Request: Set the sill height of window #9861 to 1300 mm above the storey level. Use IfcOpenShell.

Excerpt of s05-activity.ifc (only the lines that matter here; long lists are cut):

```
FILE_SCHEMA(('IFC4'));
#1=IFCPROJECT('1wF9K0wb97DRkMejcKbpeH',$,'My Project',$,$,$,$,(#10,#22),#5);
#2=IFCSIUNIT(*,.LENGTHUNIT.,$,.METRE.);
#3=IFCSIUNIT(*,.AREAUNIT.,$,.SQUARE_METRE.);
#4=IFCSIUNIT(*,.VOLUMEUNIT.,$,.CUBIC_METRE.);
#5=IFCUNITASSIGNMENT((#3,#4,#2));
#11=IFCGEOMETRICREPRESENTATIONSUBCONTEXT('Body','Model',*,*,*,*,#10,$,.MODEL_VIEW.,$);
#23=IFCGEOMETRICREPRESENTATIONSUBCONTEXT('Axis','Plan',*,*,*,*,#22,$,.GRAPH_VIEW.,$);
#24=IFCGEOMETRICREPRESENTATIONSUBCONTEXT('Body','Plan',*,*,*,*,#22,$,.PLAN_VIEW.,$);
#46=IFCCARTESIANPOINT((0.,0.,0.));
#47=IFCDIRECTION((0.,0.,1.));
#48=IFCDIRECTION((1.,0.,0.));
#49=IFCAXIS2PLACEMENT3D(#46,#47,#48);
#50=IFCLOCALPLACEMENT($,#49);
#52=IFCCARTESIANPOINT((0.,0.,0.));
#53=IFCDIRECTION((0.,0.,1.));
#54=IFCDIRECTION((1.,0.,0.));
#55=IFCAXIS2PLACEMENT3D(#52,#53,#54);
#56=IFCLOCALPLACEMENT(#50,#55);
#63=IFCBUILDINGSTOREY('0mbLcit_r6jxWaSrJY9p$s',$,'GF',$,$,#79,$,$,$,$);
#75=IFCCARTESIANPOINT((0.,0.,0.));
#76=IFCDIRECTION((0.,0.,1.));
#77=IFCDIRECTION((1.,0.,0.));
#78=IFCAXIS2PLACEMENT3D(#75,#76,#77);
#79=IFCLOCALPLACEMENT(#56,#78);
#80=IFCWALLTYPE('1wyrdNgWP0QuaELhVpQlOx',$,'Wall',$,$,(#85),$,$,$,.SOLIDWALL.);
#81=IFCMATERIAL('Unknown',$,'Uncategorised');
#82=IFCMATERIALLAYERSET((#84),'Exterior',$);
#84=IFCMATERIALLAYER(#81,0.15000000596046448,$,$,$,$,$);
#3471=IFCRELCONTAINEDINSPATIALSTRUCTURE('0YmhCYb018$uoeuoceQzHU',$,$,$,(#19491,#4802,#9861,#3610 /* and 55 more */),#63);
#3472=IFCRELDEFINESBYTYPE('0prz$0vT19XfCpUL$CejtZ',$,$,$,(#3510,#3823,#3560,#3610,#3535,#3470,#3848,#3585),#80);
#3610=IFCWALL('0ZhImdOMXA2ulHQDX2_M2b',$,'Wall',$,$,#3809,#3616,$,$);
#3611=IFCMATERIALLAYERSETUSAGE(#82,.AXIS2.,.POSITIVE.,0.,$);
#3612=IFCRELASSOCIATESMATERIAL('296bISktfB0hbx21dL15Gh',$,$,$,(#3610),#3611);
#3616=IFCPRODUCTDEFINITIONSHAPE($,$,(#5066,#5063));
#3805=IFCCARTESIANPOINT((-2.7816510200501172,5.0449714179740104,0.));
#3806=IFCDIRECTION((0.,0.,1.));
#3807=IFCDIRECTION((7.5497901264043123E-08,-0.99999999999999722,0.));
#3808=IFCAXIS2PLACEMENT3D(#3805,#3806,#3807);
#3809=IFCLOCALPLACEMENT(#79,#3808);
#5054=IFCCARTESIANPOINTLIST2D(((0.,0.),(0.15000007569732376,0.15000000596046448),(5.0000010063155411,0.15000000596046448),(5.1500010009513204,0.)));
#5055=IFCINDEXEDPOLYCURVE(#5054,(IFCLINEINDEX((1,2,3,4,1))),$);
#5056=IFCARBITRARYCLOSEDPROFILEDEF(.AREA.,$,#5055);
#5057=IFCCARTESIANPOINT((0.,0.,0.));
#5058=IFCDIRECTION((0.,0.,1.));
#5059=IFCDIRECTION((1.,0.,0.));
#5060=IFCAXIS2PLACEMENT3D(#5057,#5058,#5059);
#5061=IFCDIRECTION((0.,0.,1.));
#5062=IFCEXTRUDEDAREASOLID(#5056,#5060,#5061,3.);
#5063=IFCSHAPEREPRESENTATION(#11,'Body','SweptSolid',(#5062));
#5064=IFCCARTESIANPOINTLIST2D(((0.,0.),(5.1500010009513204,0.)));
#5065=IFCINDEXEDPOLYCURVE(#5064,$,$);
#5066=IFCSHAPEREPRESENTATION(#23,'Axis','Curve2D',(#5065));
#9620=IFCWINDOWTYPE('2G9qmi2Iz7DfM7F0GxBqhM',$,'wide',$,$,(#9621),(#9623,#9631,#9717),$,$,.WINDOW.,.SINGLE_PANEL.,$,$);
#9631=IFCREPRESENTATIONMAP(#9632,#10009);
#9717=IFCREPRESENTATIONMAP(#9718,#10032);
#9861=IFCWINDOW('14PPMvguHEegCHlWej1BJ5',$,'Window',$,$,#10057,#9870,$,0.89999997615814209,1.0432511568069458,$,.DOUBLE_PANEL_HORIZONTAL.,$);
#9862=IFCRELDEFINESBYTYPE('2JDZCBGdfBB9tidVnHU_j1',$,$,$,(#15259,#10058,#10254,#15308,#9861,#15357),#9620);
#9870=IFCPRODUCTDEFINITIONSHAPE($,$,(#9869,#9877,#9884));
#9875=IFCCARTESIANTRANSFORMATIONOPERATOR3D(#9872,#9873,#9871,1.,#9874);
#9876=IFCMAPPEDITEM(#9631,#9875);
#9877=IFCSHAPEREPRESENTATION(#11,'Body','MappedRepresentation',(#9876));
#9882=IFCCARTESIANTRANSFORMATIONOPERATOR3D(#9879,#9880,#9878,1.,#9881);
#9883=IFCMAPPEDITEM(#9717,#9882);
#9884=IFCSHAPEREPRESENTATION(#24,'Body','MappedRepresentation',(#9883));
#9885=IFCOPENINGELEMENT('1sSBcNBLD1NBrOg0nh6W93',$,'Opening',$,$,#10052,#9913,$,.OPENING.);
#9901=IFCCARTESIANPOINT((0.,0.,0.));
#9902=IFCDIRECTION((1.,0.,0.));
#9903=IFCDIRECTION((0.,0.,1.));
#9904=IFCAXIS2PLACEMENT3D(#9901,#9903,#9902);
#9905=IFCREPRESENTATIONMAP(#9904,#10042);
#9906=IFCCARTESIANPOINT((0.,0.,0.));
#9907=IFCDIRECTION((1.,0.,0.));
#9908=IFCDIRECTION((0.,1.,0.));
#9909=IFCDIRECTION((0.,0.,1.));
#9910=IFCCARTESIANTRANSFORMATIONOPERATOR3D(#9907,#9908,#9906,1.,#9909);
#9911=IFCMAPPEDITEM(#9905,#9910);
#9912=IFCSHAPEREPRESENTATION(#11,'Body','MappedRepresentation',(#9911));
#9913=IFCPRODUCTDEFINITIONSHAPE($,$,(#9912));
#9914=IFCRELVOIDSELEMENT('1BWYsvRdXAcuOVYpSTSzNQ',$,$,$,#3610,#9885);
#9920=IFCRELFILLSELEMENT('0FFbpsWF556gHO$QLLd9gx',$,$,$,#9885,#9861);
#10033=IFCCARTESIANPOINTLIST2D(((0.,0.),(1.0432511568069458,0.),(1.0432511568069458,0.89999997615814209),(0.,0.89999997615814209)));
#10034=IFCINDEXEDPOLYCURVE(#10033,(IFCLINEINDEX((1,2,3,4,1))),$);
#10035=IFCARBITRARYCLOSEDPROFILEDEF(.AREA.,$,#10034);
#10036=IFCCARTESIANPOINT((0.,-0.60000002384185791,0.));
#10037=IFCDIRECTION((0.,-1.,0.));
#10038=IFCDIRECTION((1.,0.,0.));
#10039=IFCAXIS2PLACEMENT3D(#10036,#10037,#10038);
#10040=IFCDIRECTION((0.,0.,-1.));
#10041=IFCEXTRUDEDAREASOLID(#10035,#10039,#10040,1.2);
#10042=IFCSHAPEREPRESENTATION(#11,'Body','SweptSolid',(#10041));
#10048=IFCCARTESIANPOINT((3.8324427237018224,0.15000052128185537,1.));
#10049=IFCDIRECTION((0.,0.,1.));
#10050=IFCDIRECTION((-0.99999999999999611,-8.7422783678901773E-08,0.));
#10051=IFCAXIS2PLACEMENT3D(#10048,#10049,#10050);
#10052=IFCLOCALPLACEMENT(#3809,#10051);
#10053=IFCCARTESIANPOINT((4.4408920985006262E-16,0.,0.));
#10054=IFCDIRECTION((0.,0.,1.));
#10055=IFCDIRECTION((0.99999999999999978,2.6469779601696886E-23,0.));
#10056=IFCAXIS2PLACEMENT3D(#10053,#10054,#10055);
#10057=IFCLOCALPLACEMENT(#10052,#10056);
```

```python
import numpy as np
import ifcopenshell
import ifcopenshell.api.geometry
import ifcopenshell.geom
import ifcopenshell.util.element
import ifcopenshell.util.placement
import ifcopenshell.util.shape
import ifcopenshell.util.unit

model = ifcopenshell.open("s05-activity.ifc")
unit_scale = ifcopenshell.util.unit.calculate_unit_scale(model)

window = model.by_guid("14PPMvguHEegCHlWej1BJ5")
opening = window.FillsVoids[0].RelatingOpeningElement
storey = ifcopenshell.util.element.get_container(window, ifc_class="IfcBuildingStorey")
level = ifcopenshell.util.placement.get_local_placement(storey.ObjectPlacement)[2, 3]

# The opening's origin need not be at the sill, so measure its lowest point.
shape = ifcopenshell.geom.create_shape(ifcopenshell.geom.settings(), opening)
bottom = ifcopenshell.util.shape.get_shape_bottom_elevation(shape, shape.geometry) / unit_scale
dz = level + 1.3 - bottom

shift = np.array([0.0, 0.0, dz])
# The window is placed relative to its opening, so it follows when the opening moves.
matrix = ifcopenshell.util.placement.get_local_placement(opening.ObjectPlacement)
matrix[:3, 3] += shift
ifcopenshell.api.geometry.edit_object_placement(
    model, product=opening, matrix=matrix, is_si=False, should_transform_children=True
)

print(f"moved by {dz * unit_scale:+.3f} m")

model.write("s05-activity_edited.ifc")
```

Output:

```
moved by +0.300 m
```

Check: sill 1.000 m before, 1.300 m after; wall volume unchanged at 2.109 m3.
